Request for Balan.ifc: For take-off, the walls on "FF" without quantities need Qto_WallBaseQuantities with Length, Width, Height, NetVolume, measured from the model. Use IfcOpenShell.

First a look at what the model holds.

```python
import ifcopenshell
import ifcopenshell.util.element
import ifcopenshell.util.unit

model = ifcopenshell.open("Balan.ifc")
print(model.schema)
for unit_type in ("LENGTHUNIT", "AREAUNIT", "VOLUMEUNIT"):
    print(unit_type, ifcopenshell.util.unit.calculate_unit_scale(model, unit_type))
storey = next(s for s in model.by_type("IfcBuildingStorey") if s.Name == "FF")
walls = [e for e in ifcopenshell.util.element.get_decomposition(storey) if e.is_a("IfcWall")]
for e in sorted(walls, key=lambda e: e.id()):
    print(e.id(), e.is_a(), e.Name, list(ifcopenshell.util.element.get_psets(e, qtos_only=True)), sep=" | ")
```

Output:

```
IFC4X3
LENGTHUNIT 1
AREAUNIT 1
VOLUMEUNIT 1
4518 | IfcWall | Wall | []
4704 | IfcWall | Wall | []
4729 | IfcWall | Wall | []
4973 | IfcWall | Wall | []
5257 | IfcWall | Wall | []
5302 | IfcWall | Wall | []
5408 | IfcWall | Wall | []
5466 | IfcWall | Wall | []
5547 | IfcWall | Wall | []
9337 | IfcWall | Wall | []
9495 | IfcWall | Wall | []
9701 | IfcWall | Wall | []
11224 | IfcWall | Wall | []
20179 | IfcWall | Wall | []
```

```python
import ifcopenshell
import ifcopenshell.api.pset
import ifcopenshell.geom
import ifcopenshell.util.element
import ifcopenshell.util.shape
import ifcopenshell.util.unit

model = ifcopenshell.open("Balan.ifc")
unit_scale = ifcopenshell.util.unit.calculate_unit_scale(model)
volume_scale = ifcopenshell.util.unit.calculate_unit_scale(model, "VOLUMEUNIT")
settings = ifcopenshell.geom.settings()

storey = next(s for s in model.by_type("IfcBuildingStorey") if s.Name == "FF")
walls = [e for e in ifcopenshell.util.element.get_decomposition(storey) if e.is_a("IfcWall")]

for e in sorted(walls, key=lambda e: e.id()):
    if ifcopenshell.util.element.get_psets(e, qtos_only=True, should_inherit=False):
        continue
    # Geometry comes back in metres, in the element's own axes.
    shape = ifcopenshell.geom.create_shape(settings, e)
    values = {
        "Length": ifcopenshell.util.shape.get_x(shape.geometry) / unit_scale,
        "Width": ifcopenshell.util.shape.get_y(shape.geometry) / unit_scale,
        "Height": ifcopenshell.util.shape.get_z(shape.geometry) / unit_scale,
        "NetVolume": ifcopenshell.util.shape.get_volume(shape.geometry) / volume_scale,
    }
    qto = ifcopenshell.api.pset.add_qto(model, product=e, name="Qto_WallBaseQuantities")
    ifcopenshell.api.pset.edit_qto(model, qto=qto, properties=values)
    print(e.id(), {k: round(v, 3) for k, v in values.items()})

model.write("Balan_v2.ifc")
```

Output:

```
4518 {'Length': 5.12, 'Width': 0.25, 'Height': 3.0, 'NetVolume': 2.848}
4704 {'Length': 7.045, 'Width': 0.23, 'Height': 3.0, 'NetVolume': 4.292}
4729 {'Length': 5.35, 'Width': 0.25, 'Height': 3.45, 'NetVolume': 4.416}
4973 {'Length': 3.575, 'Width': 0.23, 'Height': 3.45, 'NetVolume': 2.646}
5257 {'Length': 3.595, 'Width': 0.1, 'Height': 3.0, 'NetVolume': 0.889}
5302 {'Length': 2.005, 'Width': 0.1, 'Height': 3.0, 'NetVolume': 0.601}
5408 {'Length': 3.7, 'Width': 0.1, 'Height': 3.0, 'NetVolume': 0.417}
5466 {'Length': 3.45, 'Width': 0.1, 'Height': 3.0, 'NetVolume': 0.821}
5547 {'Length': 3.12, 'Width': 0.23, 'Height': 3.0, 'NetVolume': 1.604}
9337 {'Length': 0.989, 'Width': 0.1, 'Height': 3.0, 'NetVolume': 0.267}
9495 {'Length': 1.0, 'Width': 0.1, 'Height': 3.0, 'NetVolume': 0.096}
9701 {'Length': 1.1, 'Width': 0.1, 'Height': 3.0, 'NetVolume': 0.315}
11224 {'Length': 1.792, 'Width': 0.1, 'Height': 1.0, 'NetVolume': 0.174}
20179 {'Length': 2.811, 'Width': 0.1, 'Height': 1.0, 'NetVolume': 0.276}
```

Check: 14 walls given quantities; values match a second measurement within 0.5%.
